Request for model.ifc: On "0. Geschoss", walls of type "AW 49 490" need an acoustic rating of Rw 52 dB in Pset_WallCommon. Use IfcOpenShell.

First a look at what the model holds.

```python
import ifcopenshell
import ifcopenshell.util.element

model = ifcopenshell.open("model.ifc")
print(model.schema)
storey = next(s for s in model.by_type("IfcBuildingStorey") if s.Name == "0. Geschoss")
walls = [e for e in ifcopenshell.util.element.get_decomposition(storey) if e.is_a("IfcWall")]
seen = {}
for e in walls:
    element_type = ifcopenshell.util.element.get_type(e)
    key = (element_type.Name if element_type != e and element_type else None, ifcopenshell.util.element.get_pset(e, "Pset_WallCommon", "AcousticRating"))
    seen[key] = seen.get(key, 0) + 1
for (name, value), count in sorted(seen.items(), key=str):
    print(count, "x", name, "|", value)
```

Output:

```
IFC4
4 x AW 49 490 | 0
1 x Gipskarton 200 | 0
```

```python
import ifcopenshell
import ifcopenshell.api.pset
import ifcopenshell.util.element

model = ifcopenshell.open("model.ifc")

storey = next(s for s in model.by_type("IfcBuildingStorey") if s.Name == "0. Geschoss")
walls = [e for e in ifcopenshell.util.element.get_decomposition(storey) if e.is_a("IfcWall")]

count = 0
for e in walls:
    element_type = ifcopenshell.util.element.get_type(e)
    if element_type in (None, e) or element_type.Name != "AW 49 490":
        continue
    # add_pset returns the element's existing set when there is one.
    pset = ifcopenshell.api.pset.add_pset(model, product=e, name="Pset_WallCommon")
    ifcopenshell.api.pset.edit_pset(model, pset=pset, properties={"AcousticRating": "Rw 52 dB"})
    count += 1

print(count, "walls updated")

model.write("model_updated.ifc")
```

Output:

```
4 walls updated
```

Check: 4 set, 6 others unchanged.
